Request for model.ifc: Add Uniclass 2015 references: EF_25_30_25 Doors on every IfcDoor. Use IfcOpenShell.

First a look at what the model holds.

```python
import ifcopenshell

model = ifcopenshell.open("model.ifc")
print(model.schema)
print("classifications:", [c.Name for c in model.by_type("IfcClassification")])
for ifc_class in ("IfcDoor", "IfcRoof", "IfcStair", "IfcWall", "IfcWindow"):
    print(ifc_class, len(model.by_type(ifc_class)))
```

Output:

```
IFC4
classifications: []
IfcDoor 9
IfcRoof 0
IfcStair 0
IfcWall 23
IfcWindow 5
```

```python
import ifcopenshell
import ifcopenshell.api.classification

model = ifcopenshell.open("model.ifc")

system = ifcopenshell.api.classification.add_classification(model, classification="Uniclass 2015")

codes = {
    "IfcDoor": ("EF_25_30_25", "Doors"),
}
for ifc_class, (code, name) in codes.items():
    products = model.by_type(ifc_class)
    ifcopenshell.api.classification.add_reference(
        model, products=products, classification=system, identification=code, name=name
    )
    print(code, len(products))

model.write("model_v2.ifc")
```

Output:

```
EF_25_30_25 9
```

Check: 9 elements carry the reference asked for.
